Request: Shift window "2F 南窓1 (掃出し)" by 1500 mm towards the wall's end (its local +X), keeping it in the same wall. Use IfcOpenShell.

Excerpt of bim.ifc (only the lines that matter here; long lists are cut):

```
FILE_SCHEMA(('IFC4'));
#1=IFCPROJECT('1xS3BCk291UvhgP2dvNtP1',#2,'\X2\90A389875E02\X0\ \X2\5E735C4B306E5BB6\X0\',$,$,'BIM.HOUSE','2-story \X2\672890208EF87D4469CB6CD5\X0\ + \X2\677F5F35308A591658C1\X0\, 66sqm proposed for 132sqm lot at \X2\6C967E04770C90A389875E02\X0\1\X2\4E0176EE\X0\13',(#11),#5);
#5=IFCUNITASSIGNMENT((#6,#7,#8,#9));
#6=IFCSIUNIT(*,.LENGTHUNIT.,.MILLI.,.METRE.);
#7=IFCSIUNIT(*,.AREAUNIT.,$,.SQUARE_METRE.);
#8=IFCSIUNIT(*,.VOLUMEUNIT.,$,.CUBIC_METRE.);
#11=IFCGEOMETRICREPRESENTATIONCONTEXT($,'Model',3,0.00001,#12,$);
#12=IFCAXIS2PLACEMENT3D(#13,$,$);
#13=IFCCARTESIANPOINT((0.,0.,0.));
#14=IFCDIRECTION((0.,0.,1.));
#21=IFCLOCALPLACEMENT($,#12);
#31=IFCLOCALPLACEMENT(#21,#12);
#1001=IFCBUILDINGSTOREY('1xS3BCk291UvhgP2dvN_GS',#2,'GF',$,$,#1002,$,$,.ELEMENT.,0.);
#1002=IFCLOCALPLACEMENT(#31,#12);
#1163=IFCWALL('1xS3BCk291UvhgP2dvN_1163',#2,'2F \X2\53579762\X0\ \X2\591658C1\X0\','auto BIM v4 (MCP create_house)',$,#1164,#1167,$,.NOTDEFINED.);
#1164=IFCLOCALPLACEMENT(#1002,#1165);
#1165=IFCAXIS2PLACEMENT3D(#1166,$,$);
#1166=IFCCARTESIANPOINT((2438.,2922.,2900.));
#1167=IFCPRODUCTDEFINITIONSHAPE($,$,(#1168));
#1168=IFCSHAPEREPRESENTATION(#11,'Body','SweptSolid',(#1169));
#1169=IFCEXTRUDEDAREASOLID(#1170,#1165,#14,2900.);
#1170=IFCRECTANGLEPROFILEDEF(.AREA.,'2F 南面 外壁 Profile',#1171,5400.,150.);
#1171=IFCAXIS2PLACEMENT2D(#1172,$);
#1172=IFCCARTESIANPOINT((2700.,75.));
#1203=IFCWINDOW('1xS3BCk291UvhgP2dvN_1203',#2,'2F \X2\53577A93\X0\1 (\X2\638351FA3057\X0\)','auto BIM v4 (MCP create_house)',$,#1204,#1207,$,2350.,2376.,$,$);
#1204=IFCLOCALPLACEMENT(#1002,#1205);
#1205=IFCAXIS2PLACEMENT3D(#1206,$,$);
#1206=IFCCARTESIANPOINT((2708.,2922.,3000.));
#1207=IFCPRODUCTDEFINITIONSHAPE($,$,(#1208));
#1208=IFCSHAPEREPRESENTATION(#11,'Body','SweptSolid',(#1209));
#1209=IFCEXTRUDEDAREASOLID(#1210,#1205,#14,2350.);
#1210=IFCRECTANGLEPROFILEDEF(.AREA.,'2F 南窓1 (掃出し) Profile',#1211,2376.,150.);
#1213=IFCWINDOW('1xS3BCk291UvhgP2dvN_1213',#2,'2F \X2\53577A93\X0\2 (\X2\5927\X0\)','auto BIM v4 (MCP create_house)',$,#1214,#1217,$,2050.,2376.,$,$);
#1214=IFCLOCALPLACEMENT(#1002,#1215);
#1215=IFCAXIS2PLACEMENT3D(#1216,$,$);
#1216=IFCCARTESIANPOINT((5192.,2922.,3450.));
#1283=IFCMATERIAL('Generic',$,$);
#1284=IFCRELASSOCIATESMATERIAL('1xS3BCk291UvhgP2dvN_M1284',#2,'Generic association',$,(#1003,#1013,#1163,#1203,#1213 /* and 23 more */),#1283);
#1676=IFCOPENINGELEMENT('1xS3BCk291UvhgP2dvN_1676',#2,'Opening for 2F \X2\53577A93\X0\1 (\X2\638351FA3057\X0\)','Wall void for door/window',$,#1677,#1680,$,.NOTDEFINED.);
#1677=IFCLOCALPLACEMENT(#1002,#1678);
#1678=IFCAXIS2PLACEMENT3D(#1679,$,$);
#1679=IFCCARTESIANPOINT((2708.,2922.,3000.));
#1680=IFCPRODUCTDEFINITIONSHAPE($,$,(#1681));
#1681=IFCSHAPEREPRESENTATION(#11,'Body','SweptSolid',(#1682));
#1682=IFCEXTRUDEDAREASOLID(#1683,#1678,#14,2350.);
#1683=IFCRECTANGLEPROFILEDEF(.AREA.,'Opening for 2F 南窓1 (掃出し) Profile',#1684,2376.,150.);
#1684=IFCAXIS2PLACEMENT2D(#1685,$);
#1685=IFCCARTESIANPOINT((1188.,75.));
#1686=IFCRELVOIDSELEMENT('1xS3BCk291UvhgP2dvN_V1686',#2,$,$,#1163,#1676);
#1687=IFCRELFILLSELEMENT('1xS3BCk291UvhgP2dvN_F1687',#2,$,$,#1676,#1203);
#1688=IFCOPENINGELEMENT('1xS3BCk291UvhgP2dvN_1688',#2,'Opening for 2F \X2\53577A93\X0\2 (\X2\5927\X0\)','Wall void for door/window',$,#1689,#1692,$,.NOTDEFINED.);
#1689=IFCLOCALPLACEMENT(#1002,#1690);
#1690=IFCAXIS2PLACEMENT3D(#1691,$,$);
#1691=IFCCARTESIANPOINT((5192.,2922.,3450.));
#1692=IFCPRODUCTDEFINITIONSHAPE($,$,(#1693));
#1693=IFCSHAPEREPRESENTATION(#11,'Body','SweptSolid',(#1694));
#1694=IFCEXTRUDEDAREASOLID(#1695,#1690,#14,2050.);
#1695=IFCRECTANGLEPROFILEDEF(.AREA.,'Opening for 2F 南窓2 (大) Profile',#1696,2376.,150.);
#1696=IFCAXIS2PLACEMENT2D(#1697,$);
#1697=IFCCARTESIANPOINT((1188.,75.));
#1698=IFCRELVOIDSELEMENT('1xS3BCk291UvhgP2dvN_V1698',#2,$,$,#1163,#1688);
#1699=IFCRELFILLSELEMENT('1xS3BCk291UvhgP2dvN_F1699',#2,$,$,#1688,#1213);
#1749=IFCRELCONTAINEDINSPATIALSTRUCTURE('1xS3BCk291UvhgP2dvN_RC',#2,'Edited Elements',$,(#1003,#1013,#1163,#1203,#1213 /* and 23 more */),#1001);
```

```python
import ifcopenshell
import ifcopenshell.api.geometry
import ifcopenshell.util.placement
import ifcopenshell.util.unit

model = ifcopenshell.open("bim.ifc")
unit_scale = ifcopenshell.util.unit.calculate_unit_scale(model)

window = model.by_guid("1xS3BCk291UvhgP2dvN_1203")
opening = window.FillsVoids[0].RelatingOpeningElement
wall = opening.VoidsElements[0].RelatingBuildingElement

wall_matrix = ifcopenshell.util.placement.get_local_placement(wall.ObjectPlacement)
shift = wall_matrix[:3, 0] * 1.5 / unit_scale
before = ifcopenshell.util.placement.get_local_placement(window.ObjectPlacement)[:3, 3].copy()

# The window is not placed relative to its opening, so move both.
for product in (opening, window):
    matrix = ifcopenshell.util.placement.get_local_placement(product.ObjectPlacement)
    matrix[:3, 3] += shift
    ifcopenshell.api.geometry.edit_object_placement(model, product=product, matrix=matrix, is_si=False)

after = ifcopenshell.util.placement.get_local_placement(window.ObjectPlacement)[:3, 3]
print("window moved by", (after - before).round(3) + 0.0)

model.write("bim_v2.ifc")
```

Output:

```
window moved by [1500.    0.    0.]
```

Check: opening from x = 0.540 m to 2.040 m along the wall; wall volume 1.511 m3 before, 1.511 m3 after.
